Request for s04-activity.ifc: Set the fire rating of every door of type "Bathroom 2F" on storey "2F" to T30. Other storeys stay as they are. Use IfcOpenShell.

First a look at what the model holds.

```python
import ifcopenshell
import ifcopenshell.util.element

model = ifcopenshell.open("s04-activity.ifc")
print(model.schema)
storey = next(s for s in model.by_type("IfcBuildingStorey") if s.Name == "2F")
doors = [e for e in ifcopenshell.util.element.get_decomposition(storey) if e.is_a("IfcDoor")]
seen = {}
for e in doors:
    element_type = ifcopenshell.util.element.get_type(e)
    key = (element_type.Name if element_type != e and element_type else None, ifcopenshell.util.element.get_pset(e, "Pset_DoorCommon", "FireRating"))
    seen[key] = seen.get(key, 0) + 1
for (name, value), count in sorted(seen.items(), key=str):
    print(count, "x", name, "|", value)
```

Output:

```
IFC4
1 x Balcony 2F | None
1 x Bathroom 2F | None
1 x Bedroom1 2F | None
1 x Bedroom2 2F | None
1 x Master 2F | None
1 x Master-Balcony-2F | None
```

```python
import ifcopenshell
import ifcopenshell.api.pset
import ifcopenshell.util.element

model = ifcopenshell.open("s04-activity.ifc")

storey = next(s for s in model.by_type("IfcBuildingStorey") if s.Name == "2F")
doors = [e for e in ifcopenshell.util.element.get_decomposition(storey) if e.is_a("IfcDoor")]

count = 0
for e in doors:
    element_type = ifcopenshell.util.element.get_type(e)
    if element_type in (None, e) or element_type.Name != "Bathroom 2F":
        continue
    # add_pset returns the element's existing set when there is one.
    pset = ifcopenshell.api.pset.add_pset(model, product=e, name="Pset_DoorCommon")
    ifcopenshell.api.pset.edit_pset(model, pset=pset, properties={"FireRating": "T30"})
    count += 1

print(count, "doors updated")

model.write("s04-activity_v2.ifc")
```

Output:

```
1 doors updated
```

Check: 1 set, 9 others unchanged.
